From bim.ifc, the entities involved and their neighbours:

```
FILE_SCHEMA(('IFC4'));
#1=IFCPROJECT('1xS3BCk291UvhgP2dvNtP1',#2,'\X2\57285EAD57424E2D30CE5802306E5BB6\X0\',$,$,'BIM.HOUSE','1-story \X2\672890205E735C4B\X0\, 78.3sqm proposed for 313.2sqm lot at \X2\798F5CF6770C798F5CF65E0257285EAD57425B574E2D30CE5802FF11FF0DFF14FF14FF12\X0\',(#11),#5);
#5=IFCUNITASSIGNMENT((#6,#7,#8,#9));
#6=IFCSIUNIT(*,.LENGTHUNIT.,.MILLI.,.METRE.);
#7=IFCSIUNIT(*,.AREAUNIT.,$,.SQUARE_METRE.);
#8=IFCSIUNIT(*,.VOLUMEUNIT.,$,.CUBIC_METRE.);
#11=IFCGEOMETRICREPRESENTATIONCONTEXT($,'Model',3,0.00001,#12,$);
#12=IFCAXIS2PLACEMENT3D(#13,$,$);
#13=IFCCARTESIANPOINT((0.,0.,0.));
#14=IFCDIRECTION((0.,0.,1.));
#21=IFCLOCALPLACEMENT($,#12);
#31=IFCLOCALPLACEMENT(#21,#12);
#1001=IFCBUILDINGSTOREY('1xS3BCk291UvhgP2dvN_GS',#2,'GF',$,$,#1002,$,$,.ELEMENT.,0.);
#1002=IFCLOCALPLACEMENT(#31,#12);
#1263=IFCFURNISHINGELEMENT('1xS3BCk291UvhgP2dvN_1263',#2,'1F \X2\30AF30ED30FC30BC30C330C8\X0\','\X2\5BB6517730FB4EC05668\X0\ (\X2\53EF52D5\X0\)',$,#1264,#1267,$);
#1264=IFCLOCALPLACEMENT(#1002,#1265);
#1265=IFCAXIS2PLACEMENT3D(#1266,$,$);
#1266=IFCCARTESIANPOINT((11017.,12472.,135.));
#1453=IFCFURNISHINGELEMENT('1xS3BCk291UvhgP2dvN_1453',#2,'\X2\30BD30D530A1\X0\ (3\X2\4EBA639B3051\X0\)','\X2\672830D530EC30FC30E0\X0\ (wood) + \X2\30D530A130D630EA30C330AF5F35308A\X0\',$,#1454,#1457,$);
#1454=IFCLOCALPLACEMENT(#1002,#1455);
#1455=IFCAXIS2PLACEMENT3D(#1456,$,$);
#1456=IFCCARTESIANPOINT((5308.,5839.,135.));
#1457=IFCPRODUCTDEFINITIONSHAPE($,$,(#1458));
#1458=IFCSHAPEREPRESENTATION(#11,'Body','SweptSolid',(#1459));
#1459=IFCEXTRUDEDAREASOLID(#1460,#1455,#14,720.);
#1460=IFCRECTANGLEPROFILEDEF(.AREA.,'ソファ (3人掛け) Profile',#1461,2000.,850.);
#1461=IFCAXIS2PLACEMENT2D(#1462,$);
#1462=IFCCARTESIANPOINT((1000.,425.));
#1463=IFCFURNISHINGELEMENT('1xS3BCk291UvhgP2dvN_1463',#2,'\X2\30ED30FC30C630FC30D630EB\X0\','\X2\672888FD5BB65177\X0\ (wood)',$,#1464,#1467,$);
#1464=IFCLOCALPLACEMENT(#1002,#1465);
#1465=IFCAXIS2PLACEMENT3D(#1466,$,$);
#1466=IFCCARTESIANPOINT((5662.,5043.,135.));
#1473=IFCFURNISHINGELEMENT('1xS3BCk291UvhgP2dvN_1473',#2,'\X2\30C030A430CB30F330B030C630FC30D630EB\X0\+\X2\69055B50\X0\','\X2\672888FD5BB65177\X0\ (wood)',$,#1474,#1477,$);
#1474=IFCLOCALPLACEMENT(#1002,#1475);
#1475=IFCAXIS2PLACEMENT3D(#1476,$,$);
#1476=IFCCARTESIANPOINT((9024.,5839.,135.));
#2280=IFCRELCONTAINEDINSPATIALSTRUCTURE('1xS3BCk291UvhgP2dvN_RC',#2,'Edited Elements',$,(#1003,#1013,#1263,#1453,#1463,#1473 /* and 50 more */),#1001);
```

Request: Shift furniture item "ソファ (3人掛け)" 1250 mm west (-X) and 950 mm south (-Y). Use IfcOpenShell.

```python
import ifcopenshell
import ifcopenshell.api.geometry
import ifcopenshell.util.placement
import ifcopenshell.util.unit

model = ifcopenshell.open("bim.ifc")
unit_scale = ifcopenshell.util.unit.calculate_unit_scale(model)

item = model.by_id(1453)
matrix = ifcopenshell.util.placement.get_local_placement(item.ObjectPlacement)
matrix[0, 3] -= 1.25 / unit_scale
matrix[1, 3] -= 0.95 / unit_scale
ifcopenshell.api.geometry.edit_object_placement(model, product=item, matrix=matrix, is_si=False)

print(ifcopenshell.util.placement.get_local_placement(item.ObjectPlacement).round(3) + 0.0)

model.write("bim_updated.ifc")
```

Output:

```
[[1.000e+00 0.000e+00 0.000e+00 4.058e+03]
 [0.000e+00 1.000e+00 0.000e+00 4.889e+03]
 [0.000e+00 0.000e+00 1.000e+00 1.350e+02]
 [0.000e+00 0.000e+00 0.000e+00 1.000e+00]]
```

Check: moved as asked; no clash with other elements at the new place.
